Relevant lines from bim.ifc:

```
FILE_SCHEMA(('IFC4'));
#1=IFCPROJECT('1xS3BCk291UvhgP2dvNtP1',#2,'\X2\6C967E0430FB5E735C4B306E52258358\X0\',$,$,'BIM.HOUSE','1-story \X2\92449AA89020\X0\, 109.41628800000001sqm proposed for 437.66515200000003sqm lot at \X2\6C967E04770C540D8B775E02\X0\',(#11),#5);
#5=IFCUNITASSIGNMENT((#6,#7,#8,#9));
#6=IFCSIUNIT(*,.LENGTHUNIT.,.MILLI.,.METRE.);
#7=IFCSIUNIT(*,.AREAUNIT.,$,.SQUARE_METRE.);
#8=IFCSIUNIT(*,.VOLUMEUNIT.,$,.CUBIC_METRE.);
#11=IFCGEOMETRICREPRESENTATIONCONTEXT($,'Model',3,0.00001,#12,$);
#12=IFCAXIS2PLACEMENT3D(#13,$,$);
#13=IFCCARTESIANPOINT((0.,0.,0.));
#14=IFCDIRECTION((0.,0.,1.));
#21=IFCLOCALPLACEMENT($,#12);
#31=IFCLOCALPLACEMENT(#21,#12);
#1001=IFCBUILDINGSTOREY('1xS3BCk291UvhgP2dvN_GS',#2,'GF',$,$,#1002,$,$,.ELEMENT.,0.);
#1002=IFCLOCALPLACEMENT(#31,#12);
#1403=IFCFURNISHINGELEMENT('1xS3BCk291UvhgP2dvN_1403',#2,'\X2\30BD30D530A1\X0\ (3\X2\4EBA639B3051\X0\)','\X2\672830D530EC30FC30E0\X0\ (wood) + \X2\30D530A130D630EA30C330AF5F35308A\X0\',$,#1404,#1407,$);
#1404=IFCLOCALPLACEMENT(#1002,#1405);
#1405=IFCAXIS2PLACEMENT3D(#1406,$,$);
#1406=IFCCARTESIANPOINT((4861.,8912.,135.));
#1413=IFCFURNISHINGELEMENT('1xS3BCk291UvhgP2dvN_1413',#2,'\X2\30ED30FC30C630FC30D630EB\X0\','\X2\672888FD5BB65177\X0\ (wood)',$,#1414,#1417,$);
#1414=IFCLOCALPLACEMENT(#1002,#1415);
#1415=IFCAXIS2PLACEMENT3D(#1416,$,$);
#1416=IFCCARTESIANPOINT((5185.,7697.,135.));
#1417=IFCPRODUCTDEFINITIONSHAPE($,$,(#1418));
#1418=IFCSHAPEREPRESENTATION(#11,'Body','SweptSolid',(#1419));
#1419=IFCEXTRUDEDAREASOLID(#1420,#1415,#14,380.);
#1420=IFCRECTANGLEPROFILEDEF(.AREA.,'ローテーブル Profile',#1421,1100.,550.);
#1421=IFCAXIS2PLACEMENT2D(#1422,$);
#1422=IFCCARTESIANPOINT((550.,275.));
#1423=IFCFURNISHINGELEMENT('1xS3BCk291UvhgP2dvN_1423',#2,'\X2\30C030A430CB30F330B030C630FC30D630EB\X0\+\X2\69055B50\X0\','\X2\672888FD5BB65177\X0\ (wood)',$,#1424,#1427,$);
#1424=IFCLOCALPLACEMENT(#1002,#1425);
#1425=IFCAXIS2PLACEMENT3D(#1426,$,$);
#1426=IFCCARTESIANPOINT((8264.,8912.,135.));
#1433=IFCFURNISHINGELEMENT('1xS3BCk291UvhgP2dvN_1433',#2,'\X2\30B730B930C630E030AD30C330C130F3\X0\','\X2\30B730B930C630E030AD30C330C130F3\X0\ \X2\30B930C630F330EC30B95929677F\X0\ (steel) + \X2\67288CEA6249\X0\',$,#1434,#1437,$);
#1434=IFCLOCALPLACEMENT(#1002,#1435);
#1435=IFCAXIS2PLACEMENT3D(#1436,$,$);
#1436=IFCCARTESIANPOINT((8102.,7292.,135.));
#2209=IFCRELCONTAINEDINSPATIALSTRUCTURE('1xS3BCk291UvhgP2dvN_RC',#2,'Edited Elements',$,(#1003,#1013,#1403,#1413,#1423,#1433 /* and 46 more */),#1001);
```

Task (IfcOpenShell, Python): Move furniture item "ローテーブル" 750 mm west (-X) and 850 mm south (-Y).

```python
import ifcopenshell
import ifcopenshell.api.geometry
import ifcopenshell.util.placement
import ifcopenshell.util.unit

model = ifcopenshell.open("bim.ifc")
unit_scale = ifcopenshell.util.unit.calculate_unit_scale(model)

item = model.by_guid("1xS3BCk291UvhgP2dvN_1413")
matrix = ifcopenshell.util.placement.get_local_placement(item.ObjectPlacement)
matrix[0, 3] -= 0.75 / unit_scale
matrix[1, 3] -= 0.85 / unit_scale
ifcopenshell.api.geometry.edit_object_placement(model, product=item, matrix=matrix, is_si=False)

print(ifcopenshell.util.placement.get_local_placement(item.ObjectPlacement).round(3) + 0.0)

model.write("bim_edited.ifc")
```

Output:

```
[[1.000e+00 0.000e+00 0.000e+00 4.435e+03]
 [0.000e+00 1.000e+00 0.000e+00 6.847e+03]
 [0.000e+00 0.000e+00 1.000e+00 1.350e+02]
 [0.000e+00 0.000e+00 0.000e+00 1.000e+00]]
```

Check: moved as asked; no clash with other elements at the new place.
